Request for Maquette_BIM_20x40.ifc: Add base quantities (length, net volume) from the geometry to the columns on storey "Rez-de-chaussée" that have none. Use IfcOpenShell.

First a look at what the model holds.

```python
import ifcopenshell
import ifcopenshell.util.element
import ifcopenshell.util.unit

model = ifcopenshell.open("Maquette_BIM_20x40.ifc")
print(model.schema)
for unit_type in ("LENGTHUNIT", "AREAUNIT", "VOLUMEUNIT"):
    print(unit_type, ifcopenshell.util.unit.calculate_unit_scale(model, unit_type))
storey = next(s for s in model.by_type("IfcBuildingStorey") if s.Name == "Rez-de-chaussée")
columns = [e for e in ifcopenshell.util.element.get_decomposition(storey) if e.is_a("IfcColumn")]
for e in sorted(columns, key=lambda e: e.id()):
    print(e.id(), e.is_a(), e.Name, list(ifcopenshell.util.element.get_psets(e, qtos_only=True)), sep=" | ")
```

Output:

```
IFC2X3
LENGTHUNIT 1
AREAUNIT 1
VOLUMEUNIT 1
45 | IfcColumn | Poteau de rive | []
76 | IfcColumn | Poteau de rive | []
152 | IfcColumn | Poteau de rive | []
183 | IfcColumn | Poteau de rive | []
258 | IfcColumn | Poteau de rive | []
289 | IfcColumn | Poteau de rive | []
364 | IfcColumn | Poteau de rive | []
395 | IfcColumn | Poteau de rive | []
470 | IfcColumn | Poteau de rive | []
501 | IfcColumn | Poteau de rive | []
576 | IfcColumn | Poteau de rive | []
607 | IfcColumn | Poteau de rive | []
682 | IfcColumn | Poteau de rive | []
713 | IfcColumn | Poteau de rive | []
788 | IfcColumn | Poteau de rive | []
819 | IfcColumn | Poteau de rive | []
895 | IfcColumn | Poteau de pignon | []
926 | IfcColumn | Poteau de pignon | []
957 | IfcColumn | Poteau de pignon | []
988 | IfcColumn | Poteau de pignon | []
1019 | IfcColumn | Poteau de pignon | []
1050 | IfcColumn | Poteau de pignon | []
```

```python
import ifcopenshell
import ifcopenshell.api.pset
import ifcopenshell.geom
import ifcopenshell.util.element
import ifcopenshell.util.shape
import ifcopenshell.util.unit

model = ifcopenshell.open("Maquette_BIM_20x40.ifc")
unit_scale = ifcopenshell.util.unit.calculate_unit_scale(model)
volume_scale = ifcopenshell.util.unit.calculate_unit_scale(model, "VOLUMEUNIT")
settings = ifcopenshell.geom.settings()

storey = next(s for s in model.by_type("IfcBuildingStorey") if s.Name == "Rez-de-chaussée")
columns = [e for e in ifcopenshell.util.element.get_decomposition(storey) if e.is_a("IfcColumn")]

for e in sorted(columns, key=lambda e: e.id()):
    if ifcopenshell.util.element.get_psets(e, qtos_only=True, should_inherit=False):
        continue
    # Geometry comes back in metres, in the element's own axes.
    shape = ifcopenshell.geom.create_shape(settings, e)
    values = {
        "Length": ifcopenshell.util.shape.get_z(shape.geometry) / unit_scale,
        "NetVolume": ifcopenshell.util.shape.get_volume(shape.geometry) / volume_scale,
    }
    qto = ifcopenshell.api.pset.add_qto(model, product=e, name="BaseQuantities")
    ifcopenshell.api.pset.edit_qto(model, qto=qto, properties=values)
    print(e.id(), {k: round(v, 3) for k, v in values.items()})

model.write("Maquette_BIM_20x40_edited.ifc")
```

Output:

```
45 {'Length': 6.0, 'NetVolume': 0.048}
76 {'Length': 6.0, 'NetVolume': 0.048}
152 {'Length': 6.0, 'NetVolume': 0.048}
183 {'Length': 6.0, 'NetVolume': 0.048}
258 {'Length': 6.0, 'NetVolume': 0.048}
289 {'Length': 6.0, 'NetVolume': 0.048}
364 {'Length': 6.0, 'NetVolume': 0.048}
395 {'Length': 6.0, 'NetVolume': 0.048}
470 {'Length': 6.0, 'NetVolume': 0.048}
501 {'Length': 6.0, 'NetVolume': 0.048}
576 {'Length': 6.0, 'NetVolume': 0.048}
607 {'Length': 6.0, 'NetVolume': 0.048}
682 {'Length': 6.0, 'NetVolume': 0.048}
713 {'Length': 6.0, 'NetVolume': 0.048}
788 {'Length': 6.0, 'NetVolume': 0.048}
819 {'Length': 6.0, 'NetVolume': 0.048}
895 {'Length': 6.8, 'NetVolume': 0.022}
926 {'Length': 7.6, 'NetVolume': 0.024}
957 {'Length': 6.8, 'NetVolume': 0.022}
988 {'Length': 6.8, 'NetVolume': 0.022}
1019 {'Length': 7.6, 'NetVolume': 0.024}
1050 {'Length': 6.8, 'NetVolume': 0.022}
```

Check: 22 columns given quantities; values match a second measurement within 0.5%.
